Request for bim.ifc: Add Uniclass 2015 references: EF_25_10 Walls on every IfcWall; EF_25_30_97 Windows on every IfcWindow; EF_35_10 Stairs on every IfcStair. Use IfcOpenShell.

First a look at what the model holds.

```python
import ifcopenshell

model = ifcopenshell.open("bim.ifc")
print(model.schema)
print("classifications:", [c.Name for c in model.by_type("IfcClassification")])
for ifc_class in ("IfcDoor", "IfcRoof", "IfcStair", "IfcWall", "IfcWindow"):
    print(ifc_class, len(model.by_type(ifc_class)))
```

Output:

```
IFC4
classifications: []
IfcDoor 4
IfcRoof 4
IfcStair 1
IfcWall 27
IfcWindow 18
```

```python
import ifcopenshell
import ifcopenshell.api.classification

model = ifcopenshell.open("bim.ifc")

system = ifcopenshell.api.classification.add_classification(model, classification="Uniclass 2015")

codes = {
    "IfcWall": ("EF_25_10", "Walls"),
    "IfcWindow": ("EF_25_30_97", "Windows"),
    "IfcStair": ("EF_35_10", "Stairs"),
}
for ifc_class, (code, name) in codes.items():
    products = model.by_type(ifc_class)
    ifcopenshell.api.classification.add_reference(
        model, products=products, classification=system, identification=code, name=name
    )
    print(code, len(products))

model.write("bim_rev.ifc")
```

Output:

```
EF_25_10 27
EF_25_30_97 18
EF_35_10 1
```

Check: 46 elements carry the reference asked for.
